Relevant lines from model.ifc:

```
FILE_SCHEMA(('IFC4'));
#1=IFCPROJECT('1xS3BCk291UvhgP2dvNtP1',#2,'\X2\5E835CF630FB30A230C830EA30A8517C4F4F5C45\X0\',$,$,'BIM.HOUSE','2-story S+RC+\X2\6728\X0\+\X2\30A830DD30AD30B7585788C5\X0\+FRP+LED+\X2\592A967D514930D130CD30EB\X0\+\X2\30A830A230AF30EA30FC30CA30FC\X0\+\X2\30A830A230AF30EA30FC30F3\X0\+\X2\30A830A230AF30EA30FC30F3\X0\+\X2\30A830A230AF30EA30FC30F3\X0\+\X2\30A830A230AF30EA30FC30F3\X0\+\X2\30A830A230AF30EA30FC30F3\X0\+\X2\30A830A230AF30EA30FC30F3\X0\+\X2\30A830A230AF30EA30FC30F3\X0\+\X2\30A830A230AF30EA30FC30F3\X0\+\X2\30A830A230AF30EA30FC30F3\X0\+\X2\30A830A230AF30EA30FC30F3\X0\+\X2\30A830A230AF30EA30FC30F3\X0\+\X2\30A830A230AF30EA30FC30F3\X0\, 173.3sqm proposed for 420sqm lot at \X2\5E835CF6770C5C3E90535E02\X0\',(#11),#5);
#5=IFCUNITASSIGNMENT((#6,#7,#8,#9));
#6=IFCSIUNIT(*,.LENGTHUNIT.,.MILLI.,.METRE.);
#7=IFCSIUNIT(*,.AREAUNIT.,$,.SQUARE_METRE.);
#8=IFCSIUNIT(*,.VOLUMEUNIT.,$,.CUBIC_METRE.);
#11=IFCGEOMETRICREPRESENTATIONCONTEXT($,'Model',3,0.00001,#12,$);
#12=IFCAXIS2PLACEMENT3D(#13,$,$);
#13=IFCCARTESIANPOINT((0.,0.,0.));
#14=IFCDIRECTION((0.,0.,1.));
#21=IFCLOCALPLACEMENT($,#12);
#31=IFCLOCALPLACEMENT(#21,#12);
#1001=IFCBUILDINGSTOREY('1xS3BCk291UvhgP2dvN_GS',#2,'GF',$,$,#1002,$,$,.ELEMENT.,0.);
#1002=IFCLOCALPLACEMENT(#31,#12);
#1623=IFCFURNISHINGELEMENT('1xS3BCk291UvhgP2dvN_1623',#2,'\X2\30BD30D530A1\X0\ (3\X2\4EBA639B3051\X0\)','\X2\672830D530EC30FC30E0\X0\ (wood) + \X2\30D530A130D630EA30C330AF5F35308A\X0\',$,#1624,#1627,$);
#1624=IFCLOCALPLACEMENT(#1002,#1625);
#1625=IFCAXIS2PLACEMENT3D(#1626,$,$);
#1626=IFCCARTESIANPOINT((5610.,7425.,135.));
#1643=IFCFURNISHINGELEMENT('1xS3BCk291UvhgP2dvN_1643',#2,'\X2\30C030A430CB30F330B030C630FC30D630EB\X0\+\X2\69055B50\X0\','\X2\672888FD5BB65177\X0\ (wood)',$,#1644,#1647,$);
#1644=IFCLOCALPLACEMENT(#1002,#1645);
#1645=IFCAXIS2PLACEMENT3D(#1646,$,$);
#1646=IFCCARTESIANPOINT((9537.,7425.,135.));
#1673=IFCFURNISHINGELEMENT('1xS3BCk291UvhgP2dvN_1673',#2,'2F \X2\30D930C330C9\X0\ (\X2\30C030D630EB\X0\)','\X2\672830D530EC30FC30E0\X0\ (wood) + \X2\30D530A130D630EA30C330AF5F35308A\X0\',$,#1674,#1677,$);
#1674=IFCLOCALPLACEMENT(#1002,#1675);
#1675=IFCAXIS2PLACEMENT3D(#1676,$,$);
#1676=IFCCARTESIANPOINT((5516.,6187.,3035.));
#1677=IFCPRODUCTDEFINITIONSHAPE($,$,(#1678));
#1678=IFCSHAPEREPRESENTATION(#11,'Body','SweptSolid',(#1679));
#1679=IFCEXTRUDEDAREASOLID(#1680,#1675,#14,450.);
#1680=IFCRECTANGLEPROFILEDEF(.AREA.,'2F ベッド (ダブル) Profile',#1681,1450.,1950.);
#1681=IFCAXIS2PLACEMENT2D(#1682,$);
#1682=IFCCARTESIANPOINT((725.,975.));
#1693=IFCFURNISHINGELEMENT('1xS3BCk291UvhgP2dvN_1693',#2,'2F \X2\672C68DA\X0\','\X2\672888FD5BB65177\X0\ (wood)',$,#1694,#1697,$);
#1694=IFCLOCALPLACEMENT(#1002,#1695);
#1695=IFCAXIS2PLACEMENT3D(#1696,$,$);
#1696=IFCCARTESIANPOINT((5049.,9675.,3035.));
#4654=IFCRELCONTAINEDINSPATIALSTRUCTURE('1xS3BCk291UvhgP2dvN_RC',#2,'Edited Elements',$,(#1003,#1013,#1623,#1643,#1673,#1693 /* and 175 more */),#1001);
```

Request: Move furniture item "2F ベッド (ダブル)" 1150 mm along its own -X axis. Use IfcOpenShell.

```python
import ifcopenshell
import ifcopenshell.api.geometry
import ifcopenshell.util.placement
import ifcopenshell.util.unit

model = ifcopenshell.open("model.ifc")
unit_scale = ifcopenshell.util.unit.calculate_unit_scale(model)

item = model.by_guid("1xS3BCk291UvhgP2dvN_1673")
matrix = ifcopenshell.util.placement.get_local_placement(item.ObjectPlacement)
matrix[:3, 3] -= matrix[:3, 0] * 1.15 / unit_scale
ifcopenshell.api.geometry.edit_object_placement(model, product=item, matrix=matrix, is_si=False)

print(ifcopenshell.util.placement.get_local_placement(item.ObjectPlacement).round(3) + 0.0)

model.write("model_v2.ifc")
```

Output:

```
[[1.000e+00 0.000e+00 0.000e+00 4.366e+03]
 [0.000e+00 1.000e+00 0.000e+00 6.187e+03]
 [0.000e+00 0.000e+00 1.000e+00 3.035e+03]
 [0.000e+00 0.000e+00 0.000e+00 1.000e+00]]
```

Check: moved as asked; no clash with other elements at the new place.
